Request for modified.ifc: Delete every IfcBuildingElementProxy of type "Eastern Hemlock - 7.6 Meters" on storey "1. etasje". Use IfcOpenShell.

First a look at what the model holds.

```python
import ifcopenshell
import ifcopenshell.util.element

model = ifcopenshell.open("modified.ifc")
print(model.schema)
storey = next(s for s in model.by_type("IfcBuildingStorey") if s.Name == "1. etasje")
proxies = [e for e in ifcopenshell.util.element.get_decomposition(storey) if e.is_a("IfcBuildingElementProxy")]
seen = {}
for e in proxies:
    element_type = ifcopenshell.util.element.get_type(e)
    name = element_type.Name if element_type not in (None, e) else None
    seen[name] = seen.get(name, 0) + 1
for name, count in sorted(seen.items(), key=str):
    print(count, "x", name)
```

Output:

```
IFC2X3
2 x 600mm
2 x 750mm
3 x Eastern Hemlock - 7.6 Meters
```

```python
import ifcopenshell
import ifcopenshell.api.root
import ifcopenshell.util.element

model = ifcopenshell.open("modified.ifc")

storey = next(s for s in model.by_type("IfcBuildingStorey") if s.Name == "1. etasje")
proxies = [e for e in ifcopenshell.util.element.get_decomposition(storey) if e.is_a("IfcBuildingElementProxy")]
targets = [e for e in proxies if (t := ifcopenshell.util.element.get_type(e)) not in (None, e) and t.Name == "Eastern Hemlock - 7.6 Meters"]

for e in targets:
    ifcopenshell.api.root.remove_product(model, product=e)
print(len(targets), "removed")

model.write("modified_v2.ifc")
```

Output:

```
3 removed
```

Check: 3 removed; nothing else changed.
